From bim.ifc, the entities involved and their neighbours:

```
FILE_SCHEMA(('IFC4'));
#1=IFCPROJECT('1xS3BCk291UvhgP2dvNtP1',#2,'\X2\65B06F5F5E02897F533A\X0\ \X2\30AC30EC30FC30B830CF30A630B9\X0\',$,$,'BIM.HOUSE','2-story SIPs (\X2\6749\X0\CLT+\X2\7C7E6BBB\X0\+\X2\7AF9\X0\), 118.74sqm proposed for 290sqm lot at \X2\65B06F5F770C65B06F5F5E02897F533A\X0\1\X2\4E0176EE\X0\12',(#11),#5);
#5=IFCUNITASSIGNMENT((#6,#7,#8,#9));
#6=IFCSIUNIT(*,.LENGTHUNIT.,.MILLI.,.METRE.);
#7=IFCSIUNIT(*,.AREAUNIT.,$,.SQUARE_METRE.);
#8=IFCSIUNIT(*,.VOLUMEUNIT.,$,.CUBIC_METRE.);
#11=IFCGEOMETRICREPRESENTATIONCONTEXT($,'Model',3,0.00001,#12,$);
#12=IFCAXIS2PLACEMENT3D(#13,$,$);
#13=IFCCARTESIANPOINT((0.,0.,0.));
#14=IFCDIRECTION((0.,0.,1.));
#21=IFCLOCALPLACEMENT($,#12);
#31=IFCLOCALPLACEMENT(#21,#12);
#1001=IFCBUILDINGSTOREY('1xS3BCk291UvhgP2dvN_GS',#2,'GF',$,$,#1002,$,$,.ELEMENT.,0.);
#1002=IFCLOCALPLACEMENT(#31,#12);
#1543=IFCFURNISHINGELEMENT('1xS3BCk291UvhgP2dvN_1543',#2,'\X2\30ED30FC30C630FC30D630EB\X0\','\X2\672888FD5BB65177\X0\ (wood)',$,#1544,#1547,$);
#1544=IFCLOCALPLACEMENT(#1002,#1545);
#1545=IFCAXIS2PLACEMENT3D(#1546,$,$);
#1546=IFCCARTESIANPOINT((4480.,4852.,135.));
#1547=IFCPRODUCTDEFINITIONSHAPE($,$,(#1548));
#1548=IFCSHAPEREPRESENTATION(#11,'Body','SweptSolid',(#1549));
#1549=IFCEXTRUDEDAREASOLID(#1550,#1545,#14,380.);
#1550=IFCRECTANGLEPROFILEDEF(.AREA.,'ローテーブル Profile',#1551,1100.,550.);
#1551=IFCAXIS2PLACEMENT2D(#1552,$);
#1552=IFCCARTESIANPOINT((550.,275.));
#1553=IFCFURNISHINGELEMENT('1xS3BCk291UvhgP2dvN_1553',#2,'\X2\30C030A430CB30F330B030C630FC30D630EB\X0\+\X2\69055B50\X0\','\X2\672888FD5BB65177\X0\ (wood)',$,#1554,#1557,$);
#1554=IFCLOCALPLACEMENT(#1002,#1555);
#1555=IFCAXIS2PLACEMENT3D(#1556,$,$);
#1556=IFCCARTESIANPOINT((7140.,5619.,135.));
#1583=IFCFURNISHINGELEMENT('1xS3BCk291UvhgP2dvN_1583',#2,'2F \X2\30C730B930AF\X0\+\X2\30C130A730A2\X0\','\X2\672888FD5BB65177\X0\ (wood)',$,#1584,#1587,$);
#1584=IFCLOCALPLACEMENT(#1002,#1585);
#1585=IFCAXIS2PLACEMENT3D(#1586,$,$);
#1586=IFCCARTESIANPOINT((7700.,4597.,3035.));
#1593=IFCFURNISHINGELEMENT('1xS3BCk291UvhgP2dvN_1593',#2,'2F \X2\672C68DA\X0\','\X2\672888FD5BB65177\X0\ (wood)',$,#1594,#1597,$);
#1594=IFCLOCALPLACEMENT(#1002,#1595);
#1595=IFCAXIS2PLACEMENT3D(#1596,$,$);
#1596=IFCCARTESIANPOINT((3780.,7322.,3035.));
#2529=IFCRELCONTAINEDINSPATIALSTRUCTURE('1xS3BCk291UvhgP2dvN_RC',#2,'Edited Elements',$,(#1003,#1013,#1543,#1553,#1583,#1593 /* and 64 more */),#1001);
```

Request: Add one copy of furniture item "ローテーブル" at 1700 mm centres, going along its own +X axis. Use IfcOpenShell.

```python
import ifcopenshell
import ifcopenshell.api.geometry
import ifcopenshell.api.root
import ifcopenshell.util.element
import ifcopenshell.util.placement

model = ifcopenshell.open("bim.ifc")


def reuse_history(source, copy):
    """copy_class also copies each property set's owner history, people and application; keep the originals."""
    for rel in copy.IsDefinedBy:
        if rel.is_a("IfcRelDefinesByProperties") and (history := rel.RelatingPropertyDefinition.OwnerHistory):
            rel.RelatingPropertyDefinition.OwnerHistory = source.OwnerHistory
            ifcopenshell.util.element.remove_deep2(model, history)


source = model.by_id(1543)
base = ifcopenshell.util.placement.get_local_placement(source.ObjectPlacement)
step = base[:3, 0] * 1700.0

for i in range(1, 2):
    copy = ifcopenshell.api.root.copy_class(model, product=source)
    copy.Representation = ifcopenshell.util.element.copy_deep(
        model, source.Representation, exclude=["IfcGeometricRepresentationContext", "IfcRepresentationMap"]
    )
    reuse_history(source, copy)
    matrix = base.copy()
    matrix[:3, 3] += i * step
    print("added at", matrix[:3, 3].round(3) + 0.0)
    ifcopenshell.api.geometry.edit_object_placement(model, product=copy, matrix=matrix, is_si=False)

model.write("bim_v2.ifc")
```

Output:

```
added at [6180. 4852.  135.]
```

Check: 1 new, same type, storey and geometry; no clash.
